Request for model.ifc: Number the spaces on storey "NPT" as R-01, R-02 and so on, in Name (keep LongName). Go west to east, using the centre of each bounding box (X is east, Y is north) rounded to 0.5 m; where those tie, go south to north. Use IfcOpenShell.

First a look at what the model holds.

```python
import ifcopenshell
import ifcopenshell.util.element
import ifcopenshell.util.placement

model = ifcopenshell.open("model.ifc")
print(model.schema)
storey = next(s for s in model.by_type("IfcBuildingStorey") if s.Name == "NPT")
spaces = [e for e in ifcopenshell.util.element.get_decomposition(storey) if e.is_a("IfcSpace")]
for e in sorted(spaces, key=lambda e: e.id()):
    origin = ifcopenshell.util.placement.get_local_placement(e.ObjectPlacement)[:3, 3]
    print(e.id(), e.Name, e.LongName, origin.round(2) + 0.0, sep=" | ")
```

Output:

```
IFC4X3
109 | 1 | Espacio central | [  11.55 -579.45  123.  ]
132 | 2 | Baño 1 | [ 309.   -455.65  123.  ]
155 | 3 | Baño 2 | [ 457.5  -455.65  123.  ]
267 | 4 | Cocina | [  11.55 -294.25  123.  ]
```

```python
import ifcopenshell
import ifcopenshell.geom
import ifcopenshell.util.element
import ifcopenshell.util.shape

model = ifcopenshell.open("model.ifc")
settings = ifcopenshell.geom.settings()
settings.set("use-world-coords", True)


def centre(element):
    shape = ifcopenshell.geom.create_shape(settings, element)
    return ifcopenshell.util.shape.get_bbox_centroid(shape.geometry)


storey = next(s for s in model.by_type("IfcBuildingStorey") if s.Name == "NPT")
spaces = [e for e in ifcopenshell.util.element.get_decomposition(storey) if e.is_a("IfcSpace")]

# Insertion points can sit at a corner or the storey origin, so sort by the geometry (in metres).
centres = {e: centre(e) for e in spaces}
spaces.sort(key=lambda e: (round(centres[e][0] / 0.5), centres[e][1]))

for i, e in enumerate(spaces, start=1):
    number = f"R-{i:02d}"
    e.Name = number
    print(e.id(), number)

model.write("model_rev.ifc")
```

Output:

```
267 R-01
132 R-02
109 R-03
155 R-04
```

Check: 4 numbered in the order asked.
